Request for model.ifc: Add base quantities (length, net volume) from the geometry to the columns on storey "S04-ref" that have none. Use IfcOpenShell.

First a look at what the model holds.

```python
import ifcopenshell
import ifcopenshell.util.element
import ifcopenshell.util.unit

model = ifcopenshell.open("model.ifc")
print(model.schema)
for unit_type in ("LENGTHUNIT", "AREAUNIT", "VOLUMEUNIT"):
    print(unit_type, ifcopenshell.util.unit.calculate_unit_scale(model, unit_type))
storey = next(s for s in model.by_type("IfcBuildingStorey") if s.Name == "S04-ref")
columns = [e for e in ifcopenshell.util.element.get_decomposition(storey) if e.is_a("IfcColumn")]
for e in sorted(columns, key=lambda e: e.id()):
    print(e.id(), e.is_a(), e.Name, list(ifcopenshell.util.element.get_psets(e, qtos_only=True)), sep=" | ")
```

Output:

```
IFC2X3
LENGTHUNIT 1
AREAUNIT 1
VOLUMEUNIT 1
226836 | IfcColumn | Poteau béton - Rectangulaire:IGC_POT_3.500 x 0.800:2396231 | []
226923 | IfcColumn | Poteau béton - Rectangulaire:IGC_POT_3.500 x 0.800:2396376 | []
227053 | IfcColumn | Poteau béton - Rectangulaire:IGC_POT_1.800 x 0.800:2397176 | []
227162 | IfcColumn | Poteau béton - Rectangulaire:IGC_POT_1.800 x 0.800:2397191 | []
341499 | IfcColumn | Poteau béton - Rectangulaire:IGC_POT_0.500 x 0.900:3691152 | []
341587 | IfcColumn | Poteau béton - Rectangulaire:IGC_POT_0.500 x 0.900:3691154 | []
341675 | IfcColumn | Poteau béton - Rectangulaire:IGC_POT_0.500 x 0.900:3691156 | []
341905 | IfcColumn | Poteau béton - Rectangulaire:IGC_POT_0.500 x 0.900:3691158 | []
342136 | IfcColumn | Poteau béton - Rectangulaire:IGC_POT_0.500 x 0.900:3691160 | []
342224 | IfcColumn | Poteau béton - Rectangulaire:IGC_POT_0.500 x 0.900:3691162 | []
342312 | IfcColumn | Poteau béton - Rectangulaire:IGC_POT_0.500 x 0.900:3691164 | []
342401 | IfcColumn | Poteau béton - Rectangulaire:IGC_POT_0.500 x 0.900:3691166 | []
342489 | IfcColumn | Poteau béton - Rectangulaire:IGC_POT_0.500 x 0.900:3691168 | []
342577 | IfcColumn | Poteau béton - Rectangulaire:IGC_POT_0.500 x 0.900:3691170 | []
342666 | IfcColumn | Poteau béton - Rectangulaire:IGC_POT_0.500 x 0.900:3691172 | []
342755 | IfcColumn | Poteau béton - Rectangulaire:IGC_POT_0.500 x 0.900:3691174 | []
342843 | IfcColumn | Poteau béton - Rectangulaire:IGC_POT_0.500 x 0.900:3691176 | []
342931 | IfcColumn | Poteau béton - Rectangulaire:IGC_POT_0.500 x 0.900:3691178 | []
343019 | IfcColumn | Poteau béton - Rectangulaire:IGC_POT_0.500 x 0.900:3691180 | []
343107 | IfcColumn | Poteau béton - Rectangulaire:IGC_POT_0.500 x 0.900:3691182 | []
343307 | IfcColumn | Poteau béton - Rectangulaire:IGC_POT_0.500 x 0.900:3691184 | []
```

```python
import ifcopenshell
import ifcopenshell.api.pset
import ifcopenshell.geom
import ifcopenshell.util.element
import ifcopenshell.util.shape
import ifcopenshell.util.unit

model = ifcopenshell.open("model.ifc")
unit_scale = ifcopenshell.util.unit.calculate_unit_scale(model)
volume_scale = ifcopenshell.util.unit.calculate_unit_scale(model, "VOLUMEUNIT")
settings = ifcopenshell.geom.settings()

storey = next(s for s in model.by_type("IfcBuildingStorey") if s.Name == "S04-ref")
columns = [e for e in ifcopenshell.util.element.get_decomposition(storey) if e.is_a("IfcColumn")]

for e in sorted(columns, key=lambda e: e.id()):
    if ifcopenshell.util.element.get_psets(e, qtos_only=True, should_inherit=False):
        continue
    # Geometry comes back in metres, in the element's own axes.
    shape = ifcopenshell.geom.create_shape(settings, e)
    values = {
        "Length": ifcopenshell.util.shape.get_z(shape.geometry) / unit_scale,
        "NetVolume": ifcopenshell.util.shape.get_volume(shape.geometry) / volume_scale,
    }
    qto = ifcopenshell.api.pset.add_qto(model, product=e, name="BaseQuantities")
    ifcopenshell.api.pset.edit_qto(model, qto=qto, properties=values)
    print(e.id(), {k: round(v, 3) for k, v in values.items()})

model.write("model_updated.ifc")
```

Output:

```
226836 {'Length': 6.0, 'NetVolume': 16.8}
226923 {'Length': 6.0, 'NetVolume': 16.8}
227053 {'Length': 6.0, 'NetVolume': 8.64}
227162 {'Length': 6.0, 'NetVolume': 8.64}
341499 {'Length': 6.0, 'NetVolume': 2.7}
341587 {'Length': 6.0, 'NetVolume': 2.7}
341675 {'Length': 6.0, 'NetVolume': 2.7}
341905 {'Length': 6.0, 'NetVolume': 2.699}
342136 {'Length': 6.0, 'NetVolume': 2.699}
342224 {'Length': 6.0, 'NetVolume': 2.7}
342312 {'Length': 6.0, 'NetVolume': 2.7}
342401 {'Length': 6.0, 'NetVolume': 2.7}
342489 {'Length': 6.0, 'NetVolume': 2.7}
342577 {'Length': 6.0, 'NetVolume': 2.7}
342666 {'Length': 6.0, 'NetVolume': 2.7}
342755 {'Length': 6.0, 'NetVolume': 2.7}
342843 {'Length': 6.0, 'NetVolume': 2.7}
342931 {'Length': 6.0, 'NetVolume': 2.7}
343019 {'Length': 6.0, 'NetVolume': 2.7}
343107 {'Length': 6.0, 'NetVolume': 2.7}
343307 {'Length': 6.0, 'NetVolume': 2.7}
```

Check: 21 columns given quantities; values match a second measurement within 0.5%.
